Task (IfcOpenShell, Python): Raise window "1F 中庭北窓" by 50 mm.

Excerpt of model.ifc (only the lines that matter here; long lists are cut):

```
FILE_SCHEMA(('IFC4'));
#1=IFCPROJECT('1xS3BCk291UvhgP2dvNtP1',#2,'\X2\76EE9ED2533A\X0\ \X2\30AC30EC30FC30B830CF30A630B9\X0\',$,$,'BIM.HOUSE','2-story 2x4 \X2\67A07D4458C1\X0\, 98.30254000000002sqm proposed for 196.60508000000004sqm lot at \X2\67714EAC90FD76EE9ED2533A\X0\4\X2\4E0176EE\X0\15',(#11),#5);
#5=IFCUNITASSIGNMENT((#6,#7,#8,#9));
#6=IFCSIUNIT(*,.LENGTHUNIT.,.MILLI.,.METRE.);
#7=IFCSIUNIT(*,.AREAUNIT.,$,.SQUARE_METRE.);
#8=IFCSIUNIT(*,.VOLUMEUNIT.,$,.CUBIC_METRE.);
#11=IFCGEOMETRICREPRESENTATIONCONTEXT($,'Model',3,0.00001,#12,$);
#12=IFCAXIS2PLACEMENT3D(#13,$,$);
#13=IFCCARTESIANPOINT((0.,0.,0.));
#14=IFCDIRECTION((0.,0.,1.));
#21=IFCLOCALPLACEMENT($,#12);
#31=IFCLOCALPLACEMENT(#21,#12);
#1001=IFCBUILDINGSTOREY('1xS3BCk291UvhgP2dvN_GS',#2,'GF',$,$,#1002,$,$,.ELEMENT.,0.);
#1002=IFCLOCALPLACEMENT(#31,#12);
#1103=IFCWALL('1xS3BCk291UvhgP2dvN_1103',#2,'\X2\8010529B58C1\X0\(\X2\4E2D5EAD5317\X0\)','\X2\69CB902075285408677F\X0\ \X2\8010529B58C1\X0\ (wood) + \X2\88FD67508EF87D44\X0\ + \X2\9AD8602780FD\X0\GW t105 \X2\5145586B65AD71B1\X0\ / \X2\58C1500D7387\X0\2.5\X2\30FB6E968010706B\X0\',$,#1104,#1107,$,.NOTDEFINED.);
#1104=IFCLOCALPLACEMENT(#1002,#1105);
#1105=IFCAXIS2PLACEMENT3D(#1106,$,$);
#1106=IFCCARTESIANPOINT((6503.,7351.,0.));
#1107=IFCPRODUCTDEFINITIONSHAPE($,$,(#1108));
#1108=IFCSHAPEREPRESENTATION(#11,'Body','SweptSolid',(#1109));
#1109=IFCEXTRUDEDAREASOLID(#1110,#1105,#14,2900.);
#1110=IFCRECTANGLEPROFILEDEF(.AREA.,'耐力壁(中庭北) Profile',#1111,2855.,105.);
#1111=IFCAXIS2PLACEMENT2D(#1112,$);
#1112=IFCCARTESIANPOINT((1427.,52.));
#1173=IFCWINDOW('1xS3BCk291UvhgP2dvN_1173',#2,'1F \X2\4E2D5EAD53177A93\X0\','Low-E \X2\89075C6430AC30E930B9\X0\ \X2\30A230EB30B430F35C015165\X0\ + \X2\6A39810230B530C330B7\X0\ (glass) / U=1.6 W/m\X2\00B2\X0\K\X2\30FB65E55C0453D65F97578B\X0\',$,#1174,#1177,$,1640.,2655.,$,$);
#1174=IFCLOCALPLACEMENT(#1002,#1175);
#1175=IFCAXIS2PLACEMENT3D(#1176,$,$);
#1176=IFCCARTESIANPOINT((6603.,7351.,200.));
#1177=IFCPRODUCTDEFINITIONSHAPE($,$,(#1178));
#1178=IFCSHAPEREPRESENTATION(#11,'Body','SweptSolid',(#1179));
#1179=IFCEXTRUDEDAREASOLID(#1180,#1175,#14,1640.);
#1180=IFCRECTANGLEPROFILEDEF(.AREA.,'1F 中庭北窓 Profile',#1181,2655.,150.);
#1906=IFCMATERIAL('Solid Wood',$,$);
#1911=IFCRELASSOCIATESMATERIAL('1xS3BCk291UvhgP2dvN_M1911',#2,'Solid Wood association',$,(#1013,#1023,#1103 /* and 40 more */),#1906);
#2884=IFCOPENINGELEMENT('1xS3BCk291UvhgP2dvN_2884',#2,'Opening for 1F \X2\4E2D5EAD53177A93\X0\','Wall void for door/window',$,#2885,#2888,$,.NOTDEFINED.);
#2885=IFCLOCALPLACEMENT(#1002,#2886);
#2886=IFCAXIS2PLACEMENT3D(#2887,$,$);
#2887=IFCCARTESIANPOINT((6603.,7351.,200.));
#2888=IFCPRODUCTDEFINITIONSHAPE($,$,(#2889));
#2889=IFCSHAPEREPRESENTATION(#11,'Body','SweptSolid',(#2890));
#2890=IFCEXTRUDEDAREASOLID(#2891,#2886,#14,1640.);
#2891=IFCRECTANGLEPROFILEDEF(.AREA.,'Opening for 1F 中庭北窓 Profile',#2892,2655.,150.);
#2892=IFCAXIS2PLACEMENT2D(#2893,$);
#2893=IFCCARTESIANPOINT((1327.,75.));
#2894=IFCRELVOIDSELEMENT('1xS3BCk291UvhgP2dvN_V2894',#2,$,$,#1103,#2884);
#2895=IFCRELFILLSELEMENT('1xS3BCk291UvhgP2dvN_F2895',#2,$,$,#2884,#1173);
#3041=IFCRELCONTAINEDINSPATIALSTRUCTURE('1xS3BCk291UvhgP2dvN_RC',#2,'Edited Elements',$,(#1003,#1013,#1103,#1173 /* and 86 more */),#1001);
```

```python
import numpy as np
import ifcopenshell
import ifcopenshell.api.geometry
import ifcopenshell.util.placement
import ifcopenshell.util.unit

model = ifcopenshell.open("model.ifc")
unit_scale = ifcopenshell.util.unit.calculate_unit_scale(model)

window = model.by_guid("1xS3BCk291UvhgP2dvN_1173")
opening = window.FillsVoids[0].RelatingOpeningElement
dz = 0.05 / unit_scale

shift = np.array([0.0, 0.0, dz])
# The window is not placed relative to its opening, so move both.
for product in (opening, window):
    matrix = ifcopenshell.util.placement.get_local_placement(product.ObjectPlacement)
    matrix[:3, 3] += shift
    ifcopenshell.api.geometry.edit_object_placement(model, product=product, matrix=matrix, is_si=False)

print(f"moved by {dz * unit_scale:+.3f} m")

model.write("model_edited.ifc")
```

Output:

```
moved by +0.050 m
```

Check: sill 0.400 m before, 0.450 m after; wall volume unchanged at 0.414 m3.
